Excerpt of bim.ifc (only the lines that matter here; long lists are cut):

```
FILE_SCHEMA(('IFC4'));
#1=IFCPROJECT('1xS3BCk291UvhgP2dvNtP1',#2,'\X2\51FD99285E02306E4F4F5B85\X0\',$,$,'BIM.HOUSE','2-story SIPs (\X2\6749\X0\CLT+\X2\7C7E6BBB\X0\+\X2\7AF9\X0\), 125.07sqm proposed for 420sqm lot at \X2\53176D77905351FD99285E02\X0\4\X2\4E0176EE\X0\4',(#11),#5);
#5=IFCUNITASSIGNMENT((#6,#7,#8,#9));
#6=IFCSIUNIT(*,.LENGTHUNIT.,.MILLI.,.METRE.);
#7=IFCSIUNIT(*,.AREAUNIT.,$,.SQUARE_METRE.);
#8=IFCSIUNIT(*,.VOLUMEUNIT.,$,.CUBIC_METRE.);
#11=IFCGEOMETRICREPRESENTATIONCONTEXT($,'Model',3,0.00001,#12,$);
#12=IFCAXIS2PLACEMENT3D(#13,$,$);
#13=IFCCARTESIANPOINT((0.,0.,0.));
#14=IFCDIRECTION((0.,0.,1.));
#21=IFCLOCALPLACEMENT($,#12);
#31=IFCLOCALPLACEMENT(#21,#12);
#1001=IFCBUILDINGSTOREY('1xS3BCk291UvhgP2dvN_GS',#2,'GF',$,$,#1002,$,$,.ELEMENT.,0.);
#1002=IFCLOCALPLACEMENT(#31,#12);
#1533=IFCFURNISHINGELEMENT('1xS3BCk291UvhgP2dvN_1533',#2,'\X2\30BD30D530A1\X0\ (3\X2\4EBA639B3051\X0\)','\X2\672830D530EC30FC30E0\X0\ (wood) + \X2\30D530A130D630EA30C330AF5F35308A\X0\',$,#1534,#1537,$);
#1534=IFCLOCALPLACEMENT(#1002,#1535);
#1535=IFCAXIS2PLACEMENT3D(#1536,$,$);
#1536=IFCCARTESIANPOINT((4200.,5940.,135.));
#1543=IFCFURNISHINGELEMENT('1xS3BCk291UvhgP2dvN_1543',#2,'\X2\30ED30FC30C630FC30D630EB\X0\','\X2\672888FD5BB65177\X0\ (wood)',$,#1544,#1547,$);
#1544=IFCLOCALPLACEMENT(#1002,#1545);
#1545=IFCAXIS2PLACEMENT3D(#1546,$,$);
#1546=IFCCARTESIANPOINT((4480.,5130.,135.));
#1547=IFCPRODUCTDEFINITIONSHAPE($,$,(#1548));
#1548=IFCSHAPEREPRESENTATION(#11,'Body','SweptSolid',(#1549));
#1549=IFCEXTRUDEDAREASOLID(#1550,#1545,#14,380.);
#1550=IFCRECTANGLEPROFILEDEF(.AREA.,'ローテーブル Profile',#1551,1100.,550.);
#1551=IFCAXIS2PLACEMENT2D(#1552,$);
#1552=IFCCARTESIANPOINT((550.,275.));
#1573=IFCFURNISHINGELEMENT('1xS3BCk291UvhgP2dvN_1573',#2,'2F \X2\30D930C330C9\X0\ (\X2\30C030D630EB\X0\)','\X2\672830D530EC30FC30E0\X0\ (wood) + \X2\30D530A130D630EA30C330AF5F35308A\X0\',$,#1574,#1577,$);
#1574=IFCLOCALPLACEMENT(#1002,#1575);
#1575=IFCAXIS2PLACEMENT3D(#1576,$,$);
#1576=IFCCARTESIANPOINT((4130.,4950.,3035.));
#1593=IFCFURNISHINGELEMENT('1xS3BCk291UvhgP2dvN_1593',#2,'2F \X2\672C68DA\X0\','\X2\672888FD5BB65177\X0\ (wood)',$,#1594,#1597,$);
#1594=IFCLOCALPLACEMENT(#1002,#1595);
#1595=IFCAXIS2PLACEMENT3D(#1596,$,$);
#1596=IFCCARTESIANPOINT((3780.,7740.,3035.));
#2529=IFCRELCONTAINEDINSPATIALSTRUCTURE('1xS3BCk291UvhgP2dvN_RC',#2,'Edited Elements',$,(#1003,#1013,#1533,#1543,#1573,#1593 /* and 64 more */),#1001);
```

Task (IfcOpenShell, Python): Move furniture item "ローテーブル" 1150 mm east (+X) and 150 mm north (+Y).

```python
import ifcopenshell
import ifcopenshell.api.geometry
import ifcopenshell.util.placement

model = ifcopenshell.open("bim.ifc")

item = model.by_guid("1xS3BCk291UvhgP2dvN_1543")
matrix = ifcopenshell.util.placement.get_local_placement(item.ObjectPlacement)
matrix[0, 3] += 1150.0
matrix[1, 3] += 150.0
ifcopenshell.api.geometry.edit_object_placement(model, product=item, matrix=matrix, is_si=False)

print(ifcopenshell.util.placement.get_local_placement(item.ObjectPlacement).round(3) + 0.0)

model.write("bim_updated.ifc")
```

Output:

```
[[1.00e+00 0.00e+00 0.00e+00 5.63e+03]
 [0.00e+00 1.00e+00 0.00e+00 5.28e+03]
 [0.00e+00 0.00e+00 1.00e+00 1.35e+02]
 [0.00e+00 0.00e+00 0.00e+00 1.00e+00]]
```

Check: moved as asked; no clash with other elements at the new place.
